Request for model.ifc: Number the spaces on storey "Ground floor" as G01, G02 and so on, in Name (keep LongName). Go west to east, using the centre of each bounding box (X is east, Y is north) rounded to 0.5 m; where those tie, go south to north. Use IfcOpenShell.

First a look at what the model holds.

```python
import ifcopenshell
import ifcopenshell.util.element
import ifcopenshell.util.placement

model = ifcopenshell.open("model.ifc")
print(model.schema)
storey = next(s for s in model.by_type("IfcBuildingStorey") if s.Name == "Ground floor")
spaces = [e for e in ifcopenshell.util.element.get_decomposition(storey) if e.is_a("IfcSpace")]
for e in sorted(spaces, key=lambda e: e.id()):
    origin = ifcopenshell.util.placement.get_local_placement(e.ObjectPlacement)[:3, 3]
    print(e.id(), e.Name, e.LongName, origin.round(2) + 0.0, sep=" | ")
```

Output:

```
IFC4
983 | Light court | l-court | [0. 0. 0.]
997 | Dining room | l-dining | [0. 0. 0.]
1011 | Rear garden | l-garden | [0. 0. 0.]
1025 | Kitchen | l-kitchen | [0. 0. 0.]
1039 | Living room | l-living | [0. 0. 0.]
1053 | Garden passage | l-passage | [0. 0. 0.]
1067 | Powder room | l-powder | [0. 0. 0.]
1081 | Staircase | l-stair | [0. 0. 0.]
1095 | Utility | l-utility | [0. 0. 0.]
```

```python
import ifcopenshell
import ifcopenshell.geom
import ifcopenshell.util.element
import ifcopenshell.util.shape

model = ifcopenshell.open("model.ifc")
settings = ifcopenshell.geom.settings()
settings.set("use-world-coords", True)


def centre(element):
    shape = ifcopenshell.geom.create_shape(settings, element)
    return ifcopenshell.util.shape.get_bbox_centroid(shape.geometry)


storey = next(s for s in model.by_type("IfcBuildingStorey") if s.Name == "Ground floor")
spaces = [e for e in ifcopenshell.util.element.get_decomposition(storey) if e.is_a("IfcSpace")]

# Insertion points can sit at a corner or the storey origin, so sort by the geometry (in metres).
centres = {e: centre(e) for e in spaces}
spaces.sort(key=lambda e: (round(centres[e][0] / 0.5), centres[e][1]))

for i, e in enumerate(spaces, start=1):
    number = f"G{i:02d}"
    e.Name = number
    print(e.id(), number)

model.write("model_rev.ifc")
```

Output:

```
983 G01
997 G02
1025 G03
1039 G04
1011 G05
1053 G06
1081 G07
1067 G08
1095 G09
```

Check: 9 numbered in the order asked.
